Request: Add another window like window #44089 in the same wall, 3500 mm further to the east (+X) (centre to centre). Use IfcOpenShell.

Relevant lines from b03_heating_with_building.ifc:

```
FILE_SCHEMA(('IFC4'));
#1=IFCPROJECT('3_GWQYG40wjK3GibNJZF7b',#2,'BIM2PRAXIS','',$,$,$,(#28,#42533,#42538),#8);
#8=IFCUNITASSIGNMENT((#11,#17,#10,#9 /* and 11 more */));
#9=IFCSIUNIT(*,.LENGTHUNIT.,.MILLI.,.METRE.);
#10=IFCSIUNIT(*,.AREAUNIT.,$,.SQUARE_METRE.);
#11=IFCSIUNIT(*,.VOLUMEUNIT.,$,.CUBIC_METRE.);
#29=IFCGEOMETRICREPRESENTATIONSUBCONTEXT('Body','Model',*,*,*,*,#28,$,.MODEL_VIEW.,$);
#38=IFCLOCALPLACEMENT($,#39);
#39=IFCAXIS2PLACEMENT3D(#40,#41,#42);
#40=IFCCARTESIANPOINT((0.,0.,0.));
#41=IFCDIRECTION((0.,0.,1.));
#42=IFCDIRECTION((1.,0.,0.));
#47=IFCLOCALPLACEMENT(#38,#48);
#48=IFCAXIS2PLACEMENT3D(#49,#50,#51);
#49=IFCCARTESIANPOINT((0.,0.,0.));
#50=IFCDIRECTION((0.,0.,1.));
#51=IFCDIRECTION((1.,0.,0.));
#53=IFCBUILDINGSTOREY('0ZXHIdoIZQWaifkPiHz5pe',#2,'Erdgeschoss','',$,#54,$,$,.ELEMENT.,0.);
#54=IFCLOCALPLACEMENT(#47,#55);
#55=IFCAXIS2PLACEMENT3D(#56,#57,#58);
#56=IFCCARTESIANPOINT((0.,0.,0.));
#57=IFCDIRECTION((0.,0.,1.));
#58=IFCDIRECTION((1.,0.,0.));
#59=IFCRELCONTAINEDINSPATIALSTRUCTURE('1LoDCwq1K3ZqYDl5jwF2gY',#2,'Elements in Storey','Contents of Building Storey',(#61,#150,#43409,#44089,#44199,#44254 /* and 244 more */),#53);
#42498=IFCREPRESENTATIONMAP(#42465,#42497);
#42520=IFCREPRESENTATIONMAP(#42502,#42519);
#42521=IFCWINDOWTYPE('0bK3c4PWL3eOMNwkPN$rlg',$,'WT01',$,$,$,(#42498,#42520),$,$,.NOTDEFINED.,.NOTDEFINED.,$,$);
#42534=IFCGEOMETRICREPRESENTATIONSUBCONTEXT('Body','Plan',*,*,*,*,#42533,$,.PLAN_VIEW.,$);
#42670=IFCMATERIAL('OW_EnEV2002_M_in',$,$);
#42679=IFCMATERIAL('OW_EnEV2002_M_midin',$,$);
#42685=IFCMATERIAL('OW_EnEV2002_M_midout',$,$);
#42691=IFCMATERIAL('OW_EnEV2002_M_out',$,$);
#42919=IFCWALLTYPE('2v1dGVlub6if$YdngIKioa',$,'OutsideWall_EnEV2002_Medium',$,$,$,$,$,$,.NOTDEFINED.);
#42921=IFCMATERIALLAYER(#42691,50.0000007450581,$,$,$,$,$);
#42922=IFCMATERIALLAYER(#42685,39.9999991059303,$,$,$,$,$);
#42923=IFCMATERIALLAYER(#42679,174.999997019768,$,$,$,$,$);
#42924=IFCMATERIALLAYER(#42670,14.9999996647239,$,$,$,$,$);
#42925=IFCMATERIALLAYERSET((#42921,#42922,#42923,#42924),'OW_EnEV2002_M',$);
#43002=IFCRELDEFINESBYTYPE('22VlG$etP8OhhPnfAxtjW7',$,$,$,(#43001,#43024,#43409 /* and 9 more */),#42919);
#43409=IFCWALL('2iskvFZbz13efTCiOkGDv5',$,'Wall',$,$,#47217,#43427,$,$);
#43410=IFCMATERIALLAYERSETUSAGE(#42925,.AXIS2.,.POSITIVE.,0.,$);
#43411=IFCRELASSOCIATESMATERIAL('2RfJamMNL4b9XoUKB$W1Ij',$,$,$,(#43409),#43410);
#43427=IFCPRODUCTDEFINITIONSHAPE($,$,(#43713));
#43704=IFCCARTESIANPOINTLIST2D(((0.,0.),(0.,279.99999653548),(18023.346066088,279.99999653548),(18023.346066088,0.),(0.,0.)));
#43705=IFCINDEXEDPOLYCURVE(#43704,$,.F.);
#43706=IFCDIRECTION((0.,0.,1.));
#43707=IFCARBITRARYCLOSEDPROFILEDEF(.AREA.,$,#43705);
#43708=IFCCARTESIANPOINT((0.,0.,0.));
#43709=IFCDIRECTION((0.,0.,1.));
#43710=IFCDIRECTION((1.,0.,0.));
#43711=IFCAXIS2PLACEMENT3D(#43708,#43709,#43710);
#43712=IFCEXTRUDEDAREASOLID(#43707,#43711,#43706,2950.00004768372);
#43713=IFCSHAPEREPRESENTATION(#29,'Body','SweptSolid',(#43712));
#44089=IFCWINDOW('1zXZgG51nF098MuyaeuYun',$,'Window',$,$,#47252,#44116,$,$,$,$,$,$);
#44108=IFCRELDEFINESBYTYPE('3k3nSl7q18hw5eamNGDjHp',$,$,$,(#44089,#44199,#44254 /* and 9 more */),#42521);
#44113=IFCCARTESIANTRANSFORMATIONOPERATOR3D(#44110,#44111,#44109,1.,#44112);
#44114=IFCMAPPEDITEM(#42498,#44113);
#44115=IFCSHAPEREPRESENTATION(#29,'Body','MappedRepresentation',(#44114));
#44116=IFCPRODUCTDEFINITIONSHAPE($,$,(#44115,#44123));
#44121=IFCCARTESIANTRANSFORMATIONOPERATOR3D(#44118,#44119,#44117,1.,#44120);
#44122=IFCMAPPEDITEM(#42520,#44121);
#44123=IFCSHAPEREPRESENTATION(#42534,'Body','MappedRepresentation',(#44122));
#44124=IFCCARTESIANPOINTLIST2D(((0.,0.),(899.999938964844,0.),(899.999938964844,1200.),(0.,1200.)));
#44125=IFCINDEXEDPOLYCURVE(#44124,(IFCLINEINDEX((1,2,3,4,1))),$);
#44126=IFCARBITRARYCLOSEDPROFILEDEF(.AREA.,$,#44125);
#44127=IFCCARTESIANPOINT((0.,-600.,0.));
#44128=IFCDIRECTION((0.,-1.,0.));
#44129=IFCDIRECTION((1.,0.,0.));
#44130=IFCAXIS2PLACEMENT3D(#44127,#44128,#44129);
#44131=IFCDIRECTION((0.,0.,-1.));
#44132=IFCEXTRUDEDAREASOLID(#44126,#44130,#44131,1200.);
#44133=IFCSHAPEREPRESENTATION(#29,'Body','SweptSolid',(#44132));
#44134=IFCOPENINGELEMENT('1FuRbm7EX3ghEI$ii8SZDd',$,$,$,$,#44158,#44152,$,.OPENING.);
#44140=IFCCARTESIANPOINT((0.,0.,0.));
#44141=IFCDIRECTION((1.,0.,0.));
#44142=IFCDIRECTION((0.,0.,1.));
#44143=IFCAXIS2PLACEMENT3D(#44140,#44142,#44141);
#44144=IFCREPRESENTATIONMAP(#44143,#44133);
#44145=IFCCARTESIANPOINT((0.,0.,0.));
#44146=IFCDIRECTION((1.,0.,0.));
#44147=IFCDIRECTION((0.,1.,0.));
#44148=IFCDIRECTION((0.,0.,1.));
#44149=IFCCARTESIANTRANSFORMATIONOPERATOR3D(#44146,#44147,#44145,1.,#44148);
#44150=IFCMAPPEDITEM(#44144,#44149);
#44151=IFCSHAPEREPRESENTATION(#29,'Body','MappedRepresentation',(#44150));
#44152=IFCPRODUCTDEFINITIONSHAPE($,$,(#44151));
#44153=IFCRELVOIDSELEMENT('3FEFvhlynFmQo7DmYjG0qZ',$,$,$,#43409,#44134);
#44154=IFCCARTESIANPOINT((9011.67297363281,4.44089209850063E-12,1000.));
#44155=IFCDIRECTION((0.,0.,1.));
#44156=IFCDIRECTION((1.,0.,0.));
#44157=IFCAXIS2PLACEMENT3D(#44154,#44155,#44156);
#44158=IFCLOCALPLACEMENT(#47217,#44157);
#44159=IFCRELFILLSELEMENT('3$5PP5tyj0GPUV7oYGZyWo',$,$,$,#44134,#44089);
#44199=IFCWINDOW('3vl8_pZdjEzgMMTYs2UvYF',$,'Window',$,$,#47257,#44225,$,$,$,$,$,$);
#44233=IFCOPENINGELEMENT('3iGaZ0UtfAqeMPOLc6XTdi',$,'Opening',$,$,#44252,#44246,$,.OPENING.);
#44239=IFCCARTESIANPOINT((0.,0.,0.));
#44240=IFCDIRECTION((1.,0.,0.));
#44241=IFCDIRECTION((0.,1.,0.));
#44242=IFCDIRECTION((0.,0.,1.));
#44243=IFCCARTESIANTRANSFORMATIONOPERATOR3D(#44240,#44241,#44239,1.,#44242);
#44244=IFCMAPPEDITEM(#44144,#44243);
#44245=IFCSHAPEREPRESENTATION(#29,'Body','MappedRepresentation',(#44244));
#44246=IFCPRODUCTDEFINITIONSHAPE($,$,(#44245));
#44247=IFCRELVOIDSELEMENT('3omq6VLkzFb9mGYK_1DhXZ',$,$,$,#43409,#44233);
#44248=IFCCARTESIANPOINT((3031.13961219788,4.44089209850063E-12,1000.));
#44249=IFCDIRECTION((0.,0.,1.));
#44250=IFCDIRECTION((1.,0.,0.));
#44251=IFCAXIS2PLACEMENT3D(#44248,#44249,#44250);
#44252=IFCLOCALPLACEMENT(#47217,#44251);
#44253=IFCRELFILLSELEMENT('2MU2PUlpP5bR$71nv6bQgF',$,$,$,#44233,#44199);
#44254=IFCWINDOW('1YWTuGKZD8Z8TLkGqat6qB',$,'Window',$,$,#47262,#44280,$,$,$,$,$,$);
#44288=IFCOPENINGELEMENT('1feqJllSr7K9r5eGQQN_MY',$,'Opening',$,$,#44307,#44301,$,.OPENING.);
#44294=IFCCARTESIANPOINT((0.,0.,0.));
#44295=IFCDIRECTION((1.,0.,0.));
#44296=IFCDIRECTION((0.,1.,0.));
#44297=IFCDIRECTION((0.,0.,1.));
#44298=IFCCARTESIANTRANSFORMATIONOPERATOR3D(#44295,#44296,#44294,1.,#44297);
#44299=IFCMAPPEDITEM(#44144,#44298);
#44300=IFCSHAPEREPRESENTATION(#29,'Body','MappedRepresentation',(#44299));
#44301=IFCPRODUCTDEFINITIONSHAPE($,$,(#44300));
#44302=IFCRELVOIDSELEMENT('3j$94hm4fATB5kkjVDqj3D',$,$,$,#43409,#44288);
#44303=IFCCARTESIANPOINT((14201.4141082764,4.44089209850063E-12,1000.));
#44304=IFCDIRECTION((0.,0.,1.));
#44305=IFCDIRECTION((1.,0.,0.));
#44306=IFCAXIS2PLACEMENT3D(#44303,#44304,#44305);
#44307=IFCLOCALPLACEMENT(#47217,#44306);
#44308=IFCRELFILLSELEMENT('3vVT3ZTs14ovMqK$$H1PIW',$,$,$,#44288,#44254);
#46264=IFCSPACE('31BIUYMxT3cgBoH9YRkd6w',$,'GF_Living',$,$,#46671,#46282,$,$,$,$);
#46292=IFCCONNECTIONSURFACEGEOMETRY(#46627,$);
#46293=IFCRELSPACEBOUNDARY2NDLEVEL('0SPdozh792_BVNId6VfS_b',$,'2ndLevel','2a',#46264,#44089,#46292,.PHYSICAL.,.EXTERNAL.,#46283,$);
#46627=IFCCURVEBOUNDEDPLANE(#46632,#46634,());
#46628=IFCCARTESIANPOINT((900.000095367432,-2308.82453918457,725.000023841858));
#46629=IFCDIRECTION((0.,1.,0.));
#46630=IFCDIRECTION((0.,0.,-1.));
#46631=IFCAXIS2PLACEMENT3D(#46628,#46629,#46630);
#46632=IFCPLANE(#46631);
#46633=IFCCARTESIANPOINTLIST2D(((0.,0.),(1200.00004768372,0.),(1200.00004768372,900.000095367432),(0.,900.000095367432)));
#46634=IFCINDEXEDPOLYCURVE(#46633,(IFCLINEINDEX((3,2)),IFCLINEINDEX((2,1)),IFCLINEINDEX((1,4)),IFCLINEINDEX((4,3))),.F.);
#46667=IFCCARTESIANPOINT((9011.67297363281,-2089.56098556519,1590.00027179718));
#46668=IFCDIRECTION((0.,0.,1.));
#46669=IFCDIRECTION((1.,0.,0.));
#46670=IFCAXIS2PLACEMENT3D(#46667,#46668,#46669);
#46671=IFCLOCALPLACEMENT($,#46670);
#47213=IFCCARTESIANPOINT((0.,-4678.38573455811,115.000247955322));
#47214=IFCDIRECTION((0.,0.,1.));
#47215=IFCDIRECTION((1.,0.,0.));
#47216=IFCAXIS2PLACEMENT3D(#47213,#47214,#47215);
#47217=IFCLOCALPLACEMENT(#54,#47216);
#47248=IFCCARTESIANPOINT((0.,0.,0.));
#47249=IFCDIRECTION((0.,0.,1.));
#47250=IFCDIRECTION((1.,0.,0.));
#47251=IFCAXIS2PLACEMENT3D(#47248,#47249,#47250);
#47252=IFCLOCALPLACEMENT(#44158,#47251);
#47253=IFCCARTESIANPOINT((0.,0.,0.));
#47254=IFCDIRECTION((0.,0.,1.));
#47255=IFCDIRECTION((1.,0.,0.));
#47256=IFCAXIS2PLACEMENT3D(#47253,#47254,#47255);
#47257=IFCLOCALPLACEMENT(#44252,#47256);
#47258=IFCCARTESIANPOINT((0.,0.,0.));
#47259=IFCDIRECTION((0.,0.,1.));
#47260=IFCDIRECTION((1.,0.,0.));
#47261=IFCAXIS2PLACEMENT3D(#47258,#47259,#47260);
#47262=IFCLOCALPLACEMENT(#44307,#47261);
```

```python
import numpy as np
import ifcopenshell
import ifcopenshell.api.feature
import ifcopenshell.api.geometry
import ifcopenshell.api.root
import ifcopenshell.geom
import ifcopenshell.util.element
import ifcopenshell.util.placement
import ifcopenshell.util.shape
import ifcopenshell.util.unit

model = ifcopenshell.open("b03_heating_with_building.ifc")
unit_scale = ifcopenshell.util.unit.calculate_unit_scale(model)
settings = ifcopenshell.geom.settings()


def volume(element):
    """Net volume in cubic metres, openings subtracted."""
    shape = ifcopenshell.geom.create_shape(settings, element)
    return ifcopenshell.util.shape.get_volume(shape.geometry)


window = model.by_guid("1zXZgG51nF098MuyaeuYun")
opening = window.FillsVoids[0].RelatingOpeningElement
wall = opening.VoidsElements[0].RelatingBuildingElement
before = volume(wall)
shift = ifcopenshell.util.placement.get_local_placement(wall.ObjectPlacement)[:3, 0] * 3.5 / unit_scale

# copy_class copies the void relationship, type, container and properties, but no geometry.
new_opening = ifcopenshell.api.root.copy_class(model, product=opening)
new_opening.Representation = ifcopenshell.util.element.copy_deep(
    model, opening.Representation, exclude=["IfcGeometricRepresentationContext", "IfcRepresentationMap"]
)
new_window = ifcopenshell.api.root.copy_class(model, product=window)
new_window.Representation = ifcopenshell.util.element.copy_deep(
    model, window.Representation, exclude=["IfcGeometricRepresentationContext", "IfcRepresentationMap"]
)
ifcopenshell.api.feature.add_filling(model, opening=new_opening, element=new_window)

for old, new in ((opening, new_opening), (window, new_window)):
    matrix = ifcopenshell.util.placement.get_local_placement(old.ObjectPlacement)
    matrix[:3, 3] += shift
    ifcopenshell.api.geometry.edit_object_placement(model, product=new, matrix=matrix, is_si=False)

# The copied space boundaries still share their surfaces with the original.
for rel in new_window.ProvidesBoundaries:
    if rel.ConnectionGeometry:
        rel.ConnectionGeometry = ifcopenshell.util.element.copy_deep(model, rel.ConnectionGeometry)

# Space boundary surfaces are stored in each space's coordinates; move them too.
for rel in new_window.ProvidesBoundaries:
    if not rel.ConnectionGeometry:
        continue
    surface = rel.ConnectionGeometry.SurfaceOnRelatingElement.BasisSurface
    space_matrix = ifcopenshell.util.placement.get_local_placement(rel.RelatingSpace.ObjectPlacement)
    point = np.array(surface.Position.Location.Coordinates) + space_matrix[:3, :3].T @ shift
    surface.Position = model.createIfcAxis2Placement3D(
        model.createIfcCartesianPoint(point.tolist()), surface.Position.Axis, surface.Position.RefDirection
    )

after = volume(wall)

print(f"wall volume {before:.3f} -> {after:.3f} m3")

model.write("b03_heating_with_building_rev.ifc")
```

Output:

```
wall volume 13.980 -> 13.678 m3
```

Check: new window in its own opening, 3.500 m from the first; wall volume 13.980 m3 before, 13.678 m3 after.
